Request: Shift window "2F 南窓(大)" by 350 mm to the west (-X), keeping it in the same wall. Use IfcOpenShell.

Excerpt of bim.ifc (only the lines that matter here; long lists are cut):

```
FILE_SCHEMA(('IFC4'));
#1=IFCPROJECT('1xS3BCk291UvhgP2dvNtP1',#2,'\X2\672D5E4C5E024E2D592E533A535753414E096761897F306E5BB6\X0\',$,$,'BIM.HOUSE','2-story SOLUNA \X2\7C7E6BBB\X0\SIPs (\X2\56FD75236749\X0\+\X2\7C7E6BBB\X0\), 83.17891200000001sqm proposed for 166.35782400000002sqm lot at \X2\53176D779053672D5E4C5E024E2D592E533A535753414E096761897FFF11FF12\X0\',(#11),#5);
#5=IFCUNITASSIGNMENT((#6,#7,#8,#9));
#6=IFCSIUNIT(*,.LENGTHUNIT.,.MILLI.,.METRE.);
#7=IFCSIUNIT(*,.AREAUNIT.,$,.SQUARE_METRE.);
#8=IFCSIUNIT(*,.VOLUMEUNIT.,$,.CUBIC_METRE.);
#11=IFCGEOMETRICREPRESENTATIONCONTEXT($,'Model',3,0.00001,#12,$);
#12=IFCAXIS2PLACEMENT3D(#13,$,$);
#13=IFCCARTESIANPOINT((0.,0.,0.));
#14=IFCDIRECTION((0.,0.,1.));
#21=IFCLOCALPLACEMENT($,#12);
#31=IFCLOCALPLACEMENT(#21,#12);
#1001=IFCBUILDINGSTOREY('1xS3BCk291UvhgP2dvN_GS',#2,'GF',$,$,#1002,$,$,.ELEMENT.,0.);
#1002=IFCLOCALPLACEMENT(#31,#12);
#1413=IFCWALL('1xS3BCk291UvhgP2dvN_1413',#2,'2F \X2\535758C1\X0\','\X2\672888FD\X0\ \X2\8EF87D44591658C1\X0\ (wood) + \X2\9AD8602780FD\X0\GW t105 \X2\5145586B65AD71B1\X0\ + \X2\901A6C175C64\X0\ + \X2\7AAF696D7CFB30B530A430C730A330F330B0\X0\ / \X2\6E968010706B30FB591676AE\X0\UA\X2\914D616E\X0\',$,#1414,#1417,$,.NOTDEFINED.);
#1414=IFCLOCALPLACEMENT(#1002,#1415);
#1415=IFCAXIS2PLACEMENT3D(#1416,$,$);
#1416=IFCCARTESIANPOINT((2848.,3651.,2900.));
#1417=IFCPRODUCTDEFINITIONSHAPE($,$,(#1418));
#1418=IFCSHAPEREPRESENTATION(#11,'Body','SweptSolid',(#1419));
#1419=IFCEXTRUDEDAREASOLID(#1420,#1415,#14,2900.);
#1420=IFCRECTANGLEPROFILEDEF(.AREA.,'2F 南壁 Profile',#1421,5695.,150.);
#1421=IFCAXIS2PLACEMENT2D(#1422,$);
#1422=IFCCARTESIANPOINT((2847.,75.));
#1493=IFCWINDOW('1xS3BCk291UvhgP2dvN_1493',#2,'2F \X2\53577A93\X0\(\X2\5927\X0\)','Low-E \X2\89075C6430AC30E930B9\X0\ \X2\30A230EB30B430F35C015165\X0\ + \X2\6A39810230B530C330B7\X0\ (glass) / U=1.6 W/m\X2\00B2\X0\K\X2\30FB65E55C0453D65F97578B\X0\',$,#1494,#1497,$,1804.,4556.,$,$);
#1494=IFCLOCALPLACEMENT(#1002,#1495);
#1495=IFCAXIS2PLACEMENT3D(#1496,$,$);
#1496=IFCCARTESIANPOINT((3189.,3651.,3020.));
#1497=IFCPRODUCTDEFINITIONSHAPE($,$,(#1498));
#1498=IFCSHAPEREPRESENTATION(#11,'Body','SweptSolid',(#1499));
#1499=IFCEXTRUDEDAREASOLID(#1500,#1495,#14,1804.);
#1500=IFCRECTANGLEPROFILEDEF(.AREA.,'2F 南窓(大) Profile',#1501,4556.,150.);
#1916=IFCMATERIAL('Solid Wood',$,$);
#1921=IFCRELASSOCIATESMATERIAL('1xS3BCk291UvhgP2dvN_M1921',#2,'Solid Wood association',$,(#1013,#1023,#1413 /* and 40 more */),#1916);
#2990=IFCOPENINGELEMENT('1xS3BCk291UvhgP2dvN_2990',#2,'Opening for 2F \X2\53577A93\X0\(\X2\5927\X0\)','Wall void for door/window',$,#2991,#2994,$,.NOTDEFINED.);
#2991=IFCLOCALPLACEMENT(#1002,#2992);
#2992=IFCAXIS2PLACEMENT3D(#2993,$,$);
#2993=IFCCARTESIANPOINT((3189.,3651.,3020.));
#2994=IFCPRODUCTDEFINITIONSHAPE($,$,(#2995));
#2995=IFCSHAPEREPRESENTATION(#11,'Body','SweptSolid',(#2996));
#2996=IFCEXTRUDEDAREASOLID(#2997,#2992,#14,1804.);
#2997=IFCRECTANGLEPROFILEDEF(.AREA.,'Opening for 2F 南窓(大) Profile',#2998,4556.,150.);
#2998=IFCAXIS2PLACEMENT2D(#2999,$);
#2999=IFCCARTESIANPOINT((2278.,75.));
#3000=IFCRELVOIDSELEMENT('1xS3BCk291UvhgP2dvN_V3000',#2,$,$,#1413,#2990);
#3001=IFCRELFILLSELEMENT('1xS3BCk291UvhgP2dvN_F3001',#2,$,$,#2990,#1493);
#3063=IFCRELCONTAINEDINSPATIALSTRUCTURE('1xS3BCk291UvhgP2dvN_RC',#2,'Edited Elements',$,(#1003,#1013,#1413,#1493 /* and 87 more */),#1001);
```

```python
import ifcopenshell
import ifcopenshell.api.geometry
import ifcopenshell.util.placement
import ifcopenshell.util.unit

model = ifcopenshell.open("bim.ifc")
unit_scale = ifcopenshell.util.unit.calculate_unit_scale(model)

window = model.by_guid("1xS3BCk291UvhgP2dvN_1493")
opening = window.FillsVoids[0].RelatingOpeningElement
wall = opening.VoidsElements[0].RelatingBuildingElement

wall_matrix = ifcopenshell.util.placement.get_local_placement(wall.ObjectPlacement)
shift = wall_matrix[:3, 0] * -0.35 / unit_scale
before = ifcopenshell.util.placement.get_local_placement(window.ObjectPlacement)[:3, 3].copy()

# The window is not placed relative to its opening, so move both.
for product in (opening, window):
    matrix = ifcopenshell.util.placement.get_local_placement(product.ObjectPlacement)
    matrix[:3, 3] += shift
    ifcopenshell.api.geometry.edit_object_placement(model, product=product, matrix=matrix, is_si=False)

after = ifcopenshell.util.placement.get_local_placement(window.ObjectPlacement)[:3, 3]
print("window moved by", (after - before).round(3) + 0.0)

model.write("bim_v2.ifc")
```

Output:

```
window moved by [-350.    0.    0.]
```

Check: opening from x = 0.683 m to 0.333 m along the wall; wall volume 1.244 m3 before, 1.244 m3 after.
